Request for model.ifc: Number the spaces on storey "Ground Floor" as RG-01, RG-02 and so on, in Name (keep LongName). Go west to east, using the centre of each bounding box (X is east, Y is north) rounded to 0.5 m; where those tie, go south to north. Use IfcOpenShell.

First a look at what the model holds.

```python
import ifcopenshell
import ifcopenshell.util.element
import ifcopenshell.util.placement

model = ifcopenshell.open("model.ifc")
print(model.schema)
storey = next(s for s in model.by_type("IfcBuildingStorey") if s.Name == "Ground Floor")
spaces = [e for e in ifcopenshell.util.element.get_decomposition(storey) if e.is_a("IfcSpace")]
for e in sorted(spaces, key=lambda e: e.id()):
    origin = ifcopenshell.util.placement.get_local_placement(e.ObjectPlacement)[:3, 3]
    print(e.id(), e.Name, e.LongName, origin.round(2) + 0.0, sep=" | ")
```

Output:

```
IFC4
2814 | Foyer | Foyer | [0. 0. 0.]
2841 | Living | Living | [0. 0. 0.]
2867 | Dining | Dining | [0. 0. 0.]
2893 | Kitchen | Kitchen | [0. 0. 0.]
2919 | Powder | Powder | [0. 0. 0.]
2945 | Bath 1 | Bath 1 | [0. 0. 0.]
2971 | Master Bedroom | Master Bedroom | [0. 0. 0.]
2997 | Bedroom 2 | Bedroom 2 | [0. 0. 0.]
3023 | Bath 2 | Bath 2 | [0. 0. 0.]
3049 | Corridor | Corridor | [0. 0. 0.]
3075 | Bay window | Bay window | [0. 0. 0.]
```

```python
import ifcopenshell
import ifcopenshell.geom
import ifcopenshell.util.element
import ifcopenshell.util.shape

model = ifcopenshell.open("model.ifc")
settings = ifcopenshell.geom.settings()
settings.set("use-world-coords", True)


def centre(element):
    shape = ifcopenshell.geom.create_shape(settings, element)
    return ifcopenshell.util.shape.get_bbox_centroid(shape.geometry)


storey = next(s for s in model.by_type("IfcBuildingStorey") if s.Name == "Ground Floor")
spaces = [e for e in ifcopenshell.util.element.get_decomposition(storey) if e.is_a("IfcSpace")]

# Insertion points can sit at a corner or the storey origin, so sort by the geometry (in metres).
centres = {e: centre(e) for e in spaces}
spaces.sort(key=lambda e: (round(centres[e][0] / 0.5), centres[e][1]))

for i, e in enumerate(spaces, start=1):
    number = f"RG-{i:02d}"
    e.Name = number
    print(e.id(), number)

model.write("model_rev.ifc")
```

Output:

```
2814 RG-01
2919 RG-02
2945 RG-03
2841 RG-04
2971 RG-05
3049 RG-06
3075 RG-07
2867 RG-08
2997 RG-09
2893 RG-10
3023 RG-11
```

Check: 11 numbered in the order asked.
